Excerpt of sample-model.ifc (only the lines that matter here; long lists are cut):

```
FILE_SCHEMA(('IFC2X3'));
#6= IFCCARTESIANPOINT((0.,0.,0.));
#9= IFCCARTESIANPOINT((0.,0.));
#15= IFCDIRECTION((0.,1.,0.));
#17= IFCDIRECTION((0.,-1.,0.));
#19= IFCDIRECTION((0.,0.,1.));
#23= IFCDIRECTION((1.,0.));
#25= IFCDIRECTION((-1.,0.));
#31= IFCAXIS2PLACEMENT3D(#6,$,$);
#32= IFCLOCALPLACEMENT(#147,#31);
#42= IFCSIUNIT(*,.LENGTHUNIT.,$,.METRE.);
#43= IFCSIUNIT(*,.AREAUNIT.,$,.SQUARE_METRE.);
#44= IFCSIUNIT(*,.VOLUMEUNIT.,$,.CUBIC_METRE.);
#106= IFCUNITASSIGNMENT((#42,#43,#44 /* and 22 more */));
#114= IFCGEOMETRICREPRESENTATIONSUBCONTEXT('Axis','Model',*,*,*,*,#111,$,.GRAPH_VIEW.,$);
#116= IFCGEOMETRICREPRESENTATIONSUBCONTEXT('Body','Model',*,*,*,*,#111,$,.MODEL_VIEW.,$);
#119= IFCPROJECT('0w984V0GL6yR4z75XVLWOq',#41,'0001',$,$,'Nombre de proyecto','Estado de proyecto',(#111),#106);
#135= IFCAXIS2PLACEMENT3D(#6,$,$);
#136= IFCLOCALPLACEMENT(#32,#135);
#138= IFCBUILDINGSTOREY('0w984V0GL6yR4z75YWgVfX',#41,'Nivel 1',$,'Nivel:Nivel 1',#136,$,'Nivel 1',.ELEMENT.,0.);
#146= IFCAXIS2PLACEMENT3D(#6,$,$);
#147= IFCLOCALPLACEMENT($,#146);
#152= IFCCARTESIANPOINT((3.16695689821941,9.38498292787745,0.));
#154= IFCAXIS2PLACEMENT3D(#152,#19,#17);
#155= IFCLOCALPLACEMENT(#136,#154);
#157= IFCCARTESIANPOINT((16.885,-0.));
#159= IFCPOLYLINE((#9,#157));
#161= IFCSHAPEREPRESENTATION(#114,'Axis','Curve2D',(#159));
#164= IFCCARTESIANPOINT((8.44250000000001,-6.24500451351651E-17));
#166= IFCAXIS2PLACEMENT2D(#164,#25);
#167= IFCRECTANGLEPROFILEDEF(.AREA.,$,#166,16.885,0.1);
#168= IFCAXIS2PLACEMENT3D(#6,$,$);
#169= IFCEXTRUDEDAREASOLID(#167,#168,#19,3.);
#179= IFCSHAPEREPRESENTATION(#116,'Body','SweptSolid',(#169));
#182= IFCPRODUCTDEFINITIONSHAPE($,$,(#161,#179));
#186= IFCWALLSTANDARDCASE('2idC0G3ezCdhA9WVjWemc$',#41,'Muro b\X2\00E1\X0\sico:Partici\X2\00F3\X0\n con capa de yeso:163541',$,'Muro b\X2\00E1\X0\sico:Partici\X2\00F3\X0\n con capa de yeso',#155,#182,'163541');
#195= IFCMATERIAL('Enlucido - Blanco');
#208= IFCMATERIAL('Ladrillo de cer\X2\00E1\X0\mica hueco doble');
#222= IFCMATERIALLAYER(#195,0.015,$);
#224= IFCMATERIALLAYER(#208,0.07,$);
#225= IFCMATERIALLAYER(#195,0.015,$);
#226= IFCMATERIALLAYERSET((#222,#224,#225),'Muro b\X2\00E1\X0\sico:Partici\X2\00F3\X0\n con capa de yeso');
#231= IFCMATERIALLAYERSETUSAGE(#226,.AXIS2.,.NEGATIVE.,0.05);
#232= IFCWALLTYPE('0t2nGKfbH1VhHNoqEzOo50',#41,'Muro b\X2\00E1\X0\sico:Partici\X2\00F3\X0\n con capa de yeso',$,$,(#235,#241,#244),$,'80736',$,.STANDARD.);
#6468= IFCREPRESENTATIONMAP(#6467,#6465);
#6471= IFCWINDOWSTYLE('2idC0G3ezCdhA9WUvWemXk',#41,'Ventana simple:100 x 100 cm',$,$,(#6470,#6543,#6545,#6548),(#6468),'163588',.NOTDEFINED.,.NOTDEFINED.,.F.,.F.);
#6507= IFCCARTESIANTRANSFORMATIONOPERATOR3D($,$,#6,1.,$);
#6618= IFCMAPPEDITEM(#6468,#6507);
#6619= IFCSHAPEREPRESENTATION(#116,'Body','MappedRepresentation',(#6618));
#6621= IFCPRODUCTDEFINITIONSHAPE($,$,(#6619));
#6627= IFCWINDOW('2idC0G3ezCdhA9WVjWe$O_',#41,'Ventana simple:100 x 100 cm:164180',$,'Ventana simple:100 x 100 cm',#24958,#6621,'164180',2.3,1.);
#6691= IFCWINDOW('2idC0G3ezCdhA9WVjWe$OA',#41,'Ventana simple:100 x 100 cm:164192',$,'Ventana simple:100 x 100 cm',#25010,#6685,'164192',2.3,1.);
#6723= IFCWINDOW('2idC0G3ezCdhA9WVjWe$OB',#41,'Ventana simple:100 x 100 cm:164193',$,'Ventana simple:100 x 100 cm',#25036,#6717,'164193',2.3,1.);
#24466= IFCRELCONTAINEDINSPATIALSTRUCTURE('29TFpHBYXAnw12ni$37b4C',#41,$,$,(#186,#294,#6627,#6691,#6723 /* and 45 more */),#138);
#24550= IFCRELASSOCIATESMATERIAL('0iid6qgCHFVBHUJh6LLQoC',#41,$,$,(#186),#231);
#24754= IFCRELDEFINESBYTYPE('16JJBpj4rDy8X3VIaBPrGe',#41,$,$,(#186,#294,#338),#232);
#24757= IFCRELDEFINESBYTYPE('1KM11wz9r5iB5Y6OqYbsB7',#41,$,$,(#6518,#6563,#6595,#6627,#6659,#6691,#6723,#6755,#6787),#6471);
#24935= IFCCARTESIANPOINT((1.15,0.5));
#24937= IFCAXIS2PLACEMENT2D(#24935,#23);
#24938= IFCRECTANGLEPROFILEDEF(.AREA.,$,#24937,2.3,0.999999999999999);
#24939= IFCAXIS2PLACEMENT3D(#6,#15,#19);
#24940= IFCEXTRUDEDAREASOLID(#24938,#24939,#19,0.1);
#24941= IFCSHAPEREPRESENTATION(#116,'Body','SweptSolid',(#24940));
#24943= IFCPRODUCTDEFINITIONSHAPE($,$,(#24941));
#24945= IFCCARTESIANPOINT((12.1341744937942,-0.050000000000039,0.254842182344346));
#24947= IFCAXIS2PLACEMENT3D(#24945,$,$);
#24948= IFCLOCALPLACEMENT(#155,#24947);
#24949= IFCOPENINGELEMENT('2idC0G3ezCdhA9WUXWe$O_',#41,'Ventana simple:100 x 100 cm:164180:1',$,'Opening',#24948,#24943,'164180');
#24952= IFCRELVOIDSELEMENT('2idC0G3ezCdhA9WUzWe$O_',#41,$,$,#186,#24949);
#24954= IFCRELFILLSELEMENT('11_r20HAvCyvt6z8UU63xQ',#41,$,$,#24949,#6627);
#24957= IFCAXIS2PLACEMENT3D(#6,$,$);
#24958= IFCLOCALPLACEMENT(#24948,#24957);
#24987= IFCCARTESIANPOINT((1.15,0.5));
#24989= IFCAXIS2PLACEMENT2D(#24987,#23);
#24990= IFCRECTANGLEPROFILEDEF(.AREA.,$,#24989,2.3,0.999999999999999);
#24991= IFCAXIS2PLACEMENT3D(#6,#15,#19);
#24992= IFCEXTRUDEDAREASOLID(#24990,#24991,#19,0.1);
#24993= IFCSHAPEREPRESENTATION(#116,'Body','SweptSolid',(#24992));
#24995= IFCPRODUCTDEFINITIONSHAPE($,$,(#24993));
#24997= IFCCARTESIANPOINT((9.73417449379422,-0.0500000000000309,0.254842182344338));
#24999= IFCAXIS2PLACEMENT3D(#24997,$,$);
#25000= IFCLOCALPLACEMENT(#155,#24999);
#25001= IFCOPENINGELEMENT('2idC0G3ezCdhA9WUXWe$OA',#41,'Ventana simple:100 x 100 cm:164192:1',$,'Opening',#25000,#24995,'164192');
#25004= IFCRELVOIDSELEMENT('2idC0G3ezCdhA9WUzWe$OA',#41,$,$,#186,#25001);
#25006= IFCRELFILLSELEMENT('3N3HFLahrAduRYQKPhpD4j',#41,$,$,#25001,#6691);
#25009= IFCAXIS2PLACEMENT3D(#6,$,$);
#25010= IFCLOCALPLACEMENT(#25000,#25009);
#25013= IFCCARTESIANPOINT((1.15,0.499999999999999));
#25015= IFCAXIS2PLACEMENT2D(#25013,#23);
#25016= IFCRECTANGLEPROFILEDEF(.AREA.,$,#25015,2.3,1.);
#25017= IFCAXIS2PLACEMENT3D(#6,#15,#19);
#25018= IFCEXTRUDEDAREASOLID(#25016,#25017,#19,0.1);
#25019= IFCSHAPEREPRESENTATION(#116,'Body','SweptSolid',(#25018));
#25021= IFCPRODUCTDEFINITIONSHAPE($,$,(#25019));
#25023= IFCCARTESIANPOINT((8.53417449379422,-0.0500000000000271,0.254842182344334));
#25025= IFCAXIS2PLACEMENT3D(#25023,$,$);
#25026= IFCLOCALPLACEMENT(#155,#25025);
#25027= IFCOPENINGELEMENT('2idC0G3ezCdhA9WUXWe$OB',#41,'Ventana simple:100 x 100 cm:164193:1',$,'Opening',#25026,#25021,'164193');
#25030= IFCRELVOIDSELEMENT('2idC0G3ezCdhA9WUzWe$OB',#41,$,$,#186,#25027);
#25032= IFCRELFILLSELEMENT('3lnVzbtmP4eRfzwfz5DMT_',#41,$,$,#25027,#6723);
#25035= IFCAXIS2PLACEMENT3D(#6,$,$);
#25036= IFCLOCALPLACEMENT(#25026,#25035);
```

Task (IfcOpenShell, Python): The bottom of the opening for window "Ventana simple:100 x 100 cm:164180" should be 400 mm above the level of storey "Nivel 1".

```python
import numpy as np
import ifcopenshell
import ifcopenshell.api.geometry
import ifcopenshell.geom
import ifcopenshell.util.element
import ifcopenshell.util.placement
import ifcopenshell.util.shape
import ifcopenshell.util.unit

model = ifcopenshell.open("sample-model.ifc")
unit_scale = ifcopenshell.util.unit.calculate_unit_scale(model)

window = model.by_guid("2idC0G3ezCdhA9WVjWe$O_")
opening = window.FillsVoids[0].RelatingOpeningElement
storey = ifcopenshell.util.element.get_container(window, ifc_class="IfcBuildingStorey")
level = ifcopenshell.util.placement.get_local_placement(storey.ObjectPlacement)[2, 3]

# The opening's origin need not be at the sill, so measure its lowest point.
shape = ifcopenshell.geom.create_shape(ifcopenshell.geom.settings(), opening)
bottom = ifcopenshell.util.shape.get_shape_bottom_elevation(shape, shape.geometry) / unit_scale
dz = level + 0.4 / unit_scale - bottom

shift = np.array([0.0, 0.0, dz])
# The window is placed relative to its opening, so it follows when the opening moves.
matrix = ifcopenshell.util.placement.get_local_placement(opening.ObjectPlacement)
matrix[:3, 3] += shift
ifcopenshell.api.geometry.edit_object_placement(
    model, product=opening, matrix=matrix, is_si=False, should_transform_children=True
)

print(f"moved by {dz * unit_scale:+.3f} m")

model.write("sample-model_updated.ifc")
```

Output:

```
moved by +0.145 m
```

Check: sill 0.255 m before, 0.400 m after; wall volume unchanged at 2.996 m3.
